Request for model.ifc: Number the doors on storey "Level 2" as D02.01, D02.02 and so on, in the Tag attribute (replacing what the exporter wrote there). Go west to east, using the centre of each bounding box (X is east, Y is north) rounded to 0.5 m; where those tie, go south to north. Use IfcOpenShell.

First a look at what the model holds.

```python
import ifcopenshell
import ifcopenshell.util.element
import ifcopenshell.util.placement

model = ifcopenshell.open("model.ifc")
print(model.schema)
storey = next(s for s in model.by_type("IfcBuildingStorey") if s.Name == "Level 2")
doors = [e for e in ifcopenshell.util.element.get_decomposition(storey) if e.is_a("IfcDoor")]
for e in sorted(doors, key=lambda e: e.id()):
    origin = ifcopenshell.util.placement.get_local_placement(e.ObjectPlacement)[:3, 3]
    print(e.id(), e.Tag, e.Name, origin.round(2) + 0.0, sep=" | ")
```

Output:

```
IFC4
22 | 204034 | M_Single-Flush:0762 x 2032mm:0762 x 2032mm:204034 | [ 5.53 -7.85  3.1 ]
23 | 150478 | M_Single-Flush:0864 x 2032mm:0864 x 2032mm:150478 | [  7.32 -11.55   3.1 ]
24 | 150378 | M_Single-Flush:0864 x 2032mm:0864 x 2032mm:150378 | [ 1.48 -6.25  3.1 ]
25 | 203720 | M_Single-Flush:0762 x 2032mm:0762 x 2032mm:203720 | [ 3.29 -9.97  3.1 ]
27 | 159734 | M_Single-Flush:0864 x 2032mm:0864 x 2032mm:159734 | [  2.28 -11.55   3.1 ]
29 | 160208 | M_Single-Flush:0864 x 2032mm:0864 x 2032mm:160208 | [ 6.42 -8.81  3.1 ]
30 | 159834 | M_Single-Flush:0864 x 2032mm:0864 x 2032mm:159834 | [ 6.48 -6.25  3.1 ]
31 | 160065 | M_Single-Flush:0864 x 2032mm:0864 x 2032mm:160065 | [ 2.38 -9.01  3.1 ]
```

```python
import ifcopenshell
import ifcopenshell.geom
import ifcopenshell.util.element
import ifcopenshell.util.shape

model = ifcopenshell.open("model.ifc")
settings = ifcopenshell.geom.settings()
settings.set("use-world-coords", True)


def centre(element):
    shape = ifcopenshell.geom.create_shape(settings, element)
    return ifcopenshell.util.shape.get_bbox_centroid(shape.geometry)


storey = next(s for s in model.by_type("IfcBuildingStorey") if s.Name == "Level 2")
doors = [e for e in ifcopenshell.util.element.get_decomposition(storey) if e.is_a("IfcDoor")]

# Insertion points can sit at a corner or the storey origin, so sort by the geometry (in metres).
centres = {e: centre(e) for e in doors}
doors.sort(key=lambda e: (round(centres[e][0] / 0.5), centres[e][1]))

for i, e in enumerate(doors, start=1):
    number = f"D02.{i:02d}"
    e.Tag = number
    print(e.id(), number)

model.write("model_rev.ifc")
```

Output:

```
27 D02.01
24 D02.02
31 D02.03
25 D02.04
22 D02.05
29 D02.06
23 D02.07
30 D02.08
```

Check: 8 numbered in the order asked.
